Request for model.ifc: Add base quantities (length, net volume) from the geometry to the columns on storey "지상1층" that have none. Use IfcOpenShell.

First a look at what the model holds.

```python
import ifcopenshell
import ifcopenshell.util.element
import ifcopenshell.util.unit

model = ifcopenshell.open("model.ifc")
print(model.schema)
for unit_type in ("LENGTHUNIT", "AREAUNIT", "VOLUMEUNIT"):
    print(unit_type, ifcopenshell.util.unit.calculate_unit_scale(model, unit_type))
storey = next(s for s in model.by_type("IfcBuildingStorey") if s.Name == "지상1층")
columns = [e for e in ifcopenshell.util.element.get_decomposition(storey) if e.is_a("IfcColumn")]
for e in sorted(columns, key=lambda e: e.id()):
    print(e.id(), e.is_a(), e.Name, list(ifcopenshell.util.element.get_psets(e, qtos_only=True)), sep=" | ")
```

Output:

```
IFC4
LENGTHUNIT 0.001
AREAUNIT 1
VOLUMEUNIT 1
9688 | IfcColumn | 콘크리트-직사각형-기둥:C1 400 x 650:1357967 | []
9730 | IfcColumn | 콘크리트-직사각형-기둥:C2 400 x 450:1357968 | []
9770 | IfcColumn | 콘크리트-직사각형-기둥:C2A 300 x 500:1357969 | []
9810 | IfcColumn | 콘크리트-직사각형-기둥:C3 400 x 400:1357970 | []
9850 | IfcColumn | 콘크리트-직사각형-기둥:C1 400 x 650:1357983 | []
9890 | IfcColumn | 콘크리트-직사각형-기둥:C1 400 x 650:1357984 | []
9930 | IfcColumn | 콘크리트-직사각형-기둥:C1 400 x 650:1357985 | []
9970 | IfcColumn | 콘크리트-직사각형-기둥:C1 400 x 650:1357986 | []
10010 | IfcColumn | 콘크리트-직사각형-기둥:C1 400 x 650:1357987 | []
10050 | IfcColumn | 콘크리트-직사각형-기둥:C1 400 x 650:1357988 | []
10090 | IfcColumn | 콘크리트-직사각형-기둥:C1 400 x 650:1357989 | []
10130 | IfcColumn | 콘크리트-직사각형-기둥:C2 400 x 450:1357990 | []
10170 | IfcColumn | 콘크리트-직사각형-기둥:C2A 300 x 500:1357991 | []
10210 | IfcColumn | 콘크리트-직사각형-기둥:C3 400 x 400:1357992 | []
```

```python
import ifcopenshell
import ifcopenshell.api.pset
import ifcopenshell.geom
import ifcopenshell.util.element
import ifcopenshell.util.shape
import ifcopenshell.util.unit

model = ifcopenshell.open("model.ifc")
unit_scale = ifcopenshell.util.unit.calculate_unit_scale(model)
volume_scale = ifcopenshell.util.unit.calculate_unit_scale(model, "VOLUMEUNIT")
settings = ifcopenshell.geom.settings()

storey = next(s for s in model.by_type("IfcBuildingStorey") if s.Name == "지상1층")
columns = [e for e in ifcopenshell.util.element.get_decomposition(storey) if e.is_a("IfcColumn")]

for e in sorted(columns, key=lambda e: e.id()):
    if ifcopenshell.util.element.get_psets(e, qtos_only=True, should_inherit=False):
        continue
    # Geometry comes back in metres, in the element's own axes.
    shape = ifcopenshell.geom.create_shape(settings, e)
    values = {
        "Length": ifcopenshell.util.shape.get_z(shape.geometry) / unit_scale,
        "NetVolume": ifcopenshell.util.shape.get_volume(shape.geometry) / volume_scale,
    }
    qto = ifcopenshell.api.pset.add_qto(model, product=e, name="Qto_ColumnBaseQuantities")
    ifcopenshell.api.pset.edit_qto(model, qto=qto, properties=values)
    print(e.id(), {k: round(v, 3) for k, v in values.items()})

model.write("model_updated.ifc")
```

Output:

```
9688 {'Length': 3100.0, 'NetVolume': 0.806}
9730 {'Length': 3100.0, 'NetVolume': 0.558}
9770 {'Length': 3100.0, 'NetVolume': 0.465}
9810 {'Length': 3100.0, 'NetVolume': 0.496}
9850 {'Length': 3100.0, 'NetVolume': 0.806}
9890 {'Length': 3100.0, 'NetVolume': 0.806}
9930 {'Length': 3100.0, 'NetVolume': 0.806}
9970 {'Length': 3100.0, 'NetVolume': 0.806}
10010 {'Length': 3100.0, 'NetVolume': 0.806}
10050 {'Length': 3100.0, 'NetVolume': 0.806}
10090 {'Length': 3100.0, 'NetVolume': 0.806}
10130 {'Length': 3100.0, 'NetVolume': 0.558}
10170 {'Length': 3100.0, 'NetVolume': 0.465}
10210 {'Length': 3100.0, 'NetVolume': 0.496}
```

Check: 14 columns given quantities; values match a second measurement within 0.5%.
